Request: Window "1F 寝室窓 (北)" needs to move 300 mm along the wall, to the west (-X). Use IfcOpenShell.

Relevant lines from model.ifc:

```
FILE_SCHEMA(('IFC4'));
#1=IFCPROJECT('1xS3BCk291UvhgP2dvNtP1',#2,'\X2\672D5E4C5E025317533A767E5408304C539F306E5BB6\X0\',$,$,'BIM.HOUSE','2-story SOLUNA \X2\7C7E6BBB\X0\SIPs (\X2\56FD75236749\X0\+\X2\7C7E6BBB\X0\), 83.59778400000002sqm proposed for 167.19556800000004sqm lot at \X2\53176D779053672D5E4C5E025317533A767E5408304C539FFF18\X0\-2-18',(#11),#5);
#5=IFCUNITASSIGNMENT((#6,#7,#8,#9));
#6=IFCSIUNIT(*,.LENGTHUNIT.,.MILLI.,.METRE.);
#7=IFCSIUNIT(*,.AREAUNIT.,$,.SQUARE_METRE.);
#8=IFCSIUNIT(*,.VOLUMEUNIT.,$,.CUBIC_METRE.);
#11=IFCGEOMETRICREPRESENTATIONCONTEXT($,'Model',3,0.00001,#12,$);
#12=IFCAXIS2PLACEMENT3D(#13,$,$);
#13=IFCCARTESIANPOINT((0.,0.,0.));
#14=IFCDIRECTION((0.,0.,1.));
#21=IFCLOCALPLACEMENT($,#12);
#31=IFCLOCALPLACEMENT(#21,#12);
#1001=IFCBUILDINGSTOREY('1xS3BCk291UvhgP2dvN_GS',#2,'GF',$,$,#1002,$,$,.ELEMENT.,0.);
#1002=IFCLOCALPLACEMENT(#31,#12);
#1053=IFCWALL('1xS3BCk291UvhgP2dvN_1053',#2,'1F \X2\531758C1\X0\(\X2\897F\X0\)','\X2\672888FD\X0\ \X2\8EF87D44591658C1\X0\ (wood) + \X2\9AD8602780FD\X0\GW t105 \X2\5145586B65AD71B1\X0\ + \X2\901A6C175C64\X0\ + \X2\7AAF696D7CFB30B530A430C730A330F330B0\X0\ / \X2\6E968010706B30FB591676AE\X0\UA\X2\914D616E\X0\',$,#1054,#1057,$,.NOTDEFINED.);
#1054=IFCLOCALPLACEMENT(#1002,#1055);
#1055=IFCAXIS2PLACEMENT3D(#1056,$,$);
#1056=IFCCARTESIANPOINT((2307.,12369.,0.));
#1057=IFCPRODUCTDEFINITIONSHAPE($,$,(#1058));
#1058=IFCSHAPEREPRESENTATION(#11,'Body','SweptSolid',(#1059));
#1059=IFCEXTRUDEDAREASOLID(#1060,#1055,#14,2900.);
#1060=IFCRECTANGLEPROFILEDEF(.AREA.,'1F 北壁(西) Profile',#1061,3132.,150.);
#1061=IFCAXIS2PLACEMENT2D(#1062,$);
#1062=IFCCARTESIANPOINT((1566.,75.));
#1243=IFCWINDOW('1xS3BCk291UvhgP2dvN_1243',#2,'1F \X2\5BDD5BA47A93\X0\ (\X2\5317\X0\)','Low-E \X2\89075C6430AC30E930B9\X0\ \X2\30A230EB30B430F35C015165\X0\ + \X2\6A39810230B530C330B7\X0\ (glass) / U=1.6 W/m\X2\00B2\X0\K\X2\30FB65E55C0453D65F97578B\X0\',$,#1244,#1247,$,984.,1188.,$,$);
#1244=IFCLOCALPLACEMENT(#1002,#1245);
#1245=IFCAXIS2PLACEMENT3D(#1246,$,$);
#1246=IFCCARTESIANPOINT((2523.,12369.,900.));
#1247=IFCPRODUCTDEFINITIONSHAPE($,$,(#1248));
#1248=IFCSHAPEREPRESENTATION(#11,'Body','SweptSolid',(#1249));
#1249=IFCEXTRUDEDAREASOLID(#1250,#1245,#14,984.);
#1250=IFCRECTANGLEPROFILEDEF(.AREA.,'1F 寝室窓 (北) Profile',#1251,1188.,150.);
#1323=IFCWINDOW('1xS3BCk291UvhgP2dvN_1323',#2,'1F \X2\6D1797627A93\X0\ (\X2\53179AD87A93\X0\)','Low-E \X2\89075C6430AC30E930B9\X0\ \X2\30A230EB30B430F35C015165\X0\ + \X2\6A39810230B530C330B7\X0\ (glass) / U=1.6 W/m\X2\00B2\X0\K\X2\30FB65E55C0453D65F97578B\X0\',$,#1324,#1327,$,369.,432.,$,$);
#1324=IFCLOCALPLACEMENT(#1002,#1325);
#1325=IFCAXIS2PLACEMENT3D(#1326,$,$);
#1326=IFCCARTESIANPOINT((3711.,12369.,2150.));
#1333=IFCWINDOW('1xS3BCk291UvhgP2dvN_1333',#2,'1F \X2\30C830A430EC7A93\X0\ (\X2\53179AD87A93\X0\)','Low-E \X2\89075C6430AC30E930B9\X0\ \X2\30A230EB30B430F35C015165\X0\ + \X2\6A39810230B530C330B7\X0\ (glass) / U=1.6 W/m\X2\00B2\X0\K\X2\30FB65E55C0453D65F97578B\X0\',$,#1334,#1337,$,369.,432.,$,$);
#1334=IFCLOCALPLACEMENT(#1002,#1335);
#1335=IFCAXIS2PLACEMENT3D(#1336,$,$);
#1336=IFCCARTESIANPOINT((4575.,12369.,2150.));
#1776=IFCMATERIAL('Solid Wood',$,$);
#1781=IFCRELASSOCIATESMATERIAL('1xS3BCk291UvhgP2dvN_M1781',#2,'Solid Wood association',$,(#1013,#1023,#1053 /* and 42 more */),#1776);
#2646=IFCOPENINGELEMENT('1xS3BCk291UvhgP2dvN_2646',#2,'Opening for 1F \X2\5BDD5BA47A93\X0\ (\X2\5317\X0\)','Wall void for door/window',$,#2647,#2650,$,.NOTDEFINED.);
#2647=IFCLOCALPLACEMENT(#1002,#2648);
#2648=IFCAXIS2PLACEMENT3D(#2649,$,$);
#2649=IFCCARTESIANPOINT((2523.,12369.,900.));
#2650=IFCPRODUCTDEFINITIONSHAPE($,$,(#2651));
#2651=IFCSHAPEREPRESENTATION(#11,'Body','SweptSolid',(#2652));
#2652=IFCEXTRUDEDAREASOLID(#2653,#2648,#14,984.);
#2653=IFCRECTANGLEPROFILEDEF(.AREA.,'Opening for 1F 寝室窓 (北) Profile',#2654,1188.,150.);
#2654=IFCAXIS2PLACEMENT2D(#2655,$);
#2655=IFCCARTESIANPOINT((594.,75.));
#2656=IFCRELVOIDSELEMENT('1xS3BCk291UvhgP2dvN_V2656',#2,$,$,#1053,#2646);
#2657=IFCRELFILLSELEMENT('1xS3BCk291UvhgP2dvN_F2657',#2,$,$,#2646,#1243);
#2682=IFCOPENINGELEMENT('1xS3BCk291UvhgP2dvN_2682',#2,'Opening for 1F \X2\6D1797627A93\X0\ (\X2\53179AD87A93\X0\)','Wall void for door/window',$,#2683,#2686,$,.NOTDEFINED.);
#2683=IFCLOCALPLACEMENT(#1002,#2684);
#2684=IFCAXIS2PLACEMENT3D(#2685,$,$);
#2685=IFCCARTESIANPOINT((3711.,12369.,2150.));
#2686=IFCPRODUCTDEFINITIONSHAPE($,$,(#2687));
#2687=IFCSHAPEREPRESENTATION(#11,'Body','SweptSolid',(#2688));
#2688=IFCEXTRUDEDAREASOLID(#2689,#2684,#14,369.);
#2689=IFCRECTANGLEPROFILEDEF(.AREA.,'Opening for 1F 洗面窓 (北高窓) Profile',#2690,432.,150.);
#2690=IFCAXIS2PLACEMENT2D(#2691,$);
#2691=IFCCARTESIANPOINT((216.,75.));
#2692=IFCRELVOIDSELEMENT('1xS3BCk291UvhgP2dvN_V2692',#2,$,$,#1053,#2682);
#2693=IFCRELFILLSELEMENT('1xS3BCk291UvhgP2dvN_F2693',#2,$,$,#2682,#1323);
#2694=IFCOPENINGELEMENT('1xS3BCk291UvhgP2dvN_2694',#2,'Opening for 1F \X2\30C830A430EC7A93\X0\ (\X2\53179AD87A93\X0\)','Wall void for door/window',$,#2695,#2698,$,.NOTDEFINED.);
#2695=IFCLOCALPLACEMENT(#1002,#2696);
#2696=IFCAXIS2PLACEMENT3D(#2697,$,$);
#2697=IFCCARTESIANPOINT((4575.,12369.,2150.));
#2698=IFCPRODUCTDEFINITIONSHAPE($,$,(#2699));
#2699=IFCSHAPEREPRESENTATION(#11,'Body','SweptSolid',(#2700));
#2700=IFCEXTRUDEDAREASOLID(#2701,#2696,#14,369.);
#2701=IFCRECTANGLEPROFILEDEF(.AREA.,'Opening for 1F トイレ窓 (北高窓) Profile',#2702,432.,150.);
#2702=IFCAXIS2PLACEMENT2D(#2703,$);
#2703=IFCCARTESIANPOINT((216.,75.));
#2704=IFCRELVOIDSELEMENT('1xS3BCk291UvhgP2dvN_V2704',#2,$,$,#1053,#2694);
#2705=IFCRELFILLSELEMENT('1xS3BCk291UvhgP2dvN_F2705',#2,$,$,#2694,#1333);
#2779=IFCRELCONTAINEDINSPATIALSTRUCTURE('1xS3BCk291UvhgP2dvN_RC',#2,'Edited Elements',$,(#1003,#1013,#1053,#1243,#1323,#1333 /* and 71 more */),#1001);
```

```python
import ifcopenshell
import ifcopenshell.api.geometry
import ifcopenshell.util.placement
import ifcopenshell.util.unit

model = ifcopenshell.open("model.ifc")
unit_scale = ifcopenshell.util.unit.calculate_unit_scale(model)

window = model.by_guid("1xS3BCk291UvhgP2dvN_1243")
opening = window.FillsVoids[0].RelatingOpeningElement
wall = opening.VoidsElements[0].RelatingBuildingElement

wall_matrix = ifcopenshell.util.placement.get_local_placement(wall.ObjectPlacement)
shift = wall_matrix[:3, 0] * -0.3 / unit_scale
before = ifcopenshell.util.placement.get_local_placement(window.ObjectPlacement)[:3, 3].copy()

# The window is not placed relative to its opening, so move both.
for product in (opening, window):
    matrix = ifcopenshell.util.placement.get_local_placement(product.ObjectPlacement)
    matrix[:3, 3] += shift
    ifcopenshell.api.geometry.edit_object_placement(model, product=product, matrix=matrix, is_si=False)

after = ifcopenshell.util.placement.get_local_placement(window.ObjectPlacement)[:3, 3]
print("window moved by", (after - before).round(3) + 0.0)

model.write("model-out.ifc")
```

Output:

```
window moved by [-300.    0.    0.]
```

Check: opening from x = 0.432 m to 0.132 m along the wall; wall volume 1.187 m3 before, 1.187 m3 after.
